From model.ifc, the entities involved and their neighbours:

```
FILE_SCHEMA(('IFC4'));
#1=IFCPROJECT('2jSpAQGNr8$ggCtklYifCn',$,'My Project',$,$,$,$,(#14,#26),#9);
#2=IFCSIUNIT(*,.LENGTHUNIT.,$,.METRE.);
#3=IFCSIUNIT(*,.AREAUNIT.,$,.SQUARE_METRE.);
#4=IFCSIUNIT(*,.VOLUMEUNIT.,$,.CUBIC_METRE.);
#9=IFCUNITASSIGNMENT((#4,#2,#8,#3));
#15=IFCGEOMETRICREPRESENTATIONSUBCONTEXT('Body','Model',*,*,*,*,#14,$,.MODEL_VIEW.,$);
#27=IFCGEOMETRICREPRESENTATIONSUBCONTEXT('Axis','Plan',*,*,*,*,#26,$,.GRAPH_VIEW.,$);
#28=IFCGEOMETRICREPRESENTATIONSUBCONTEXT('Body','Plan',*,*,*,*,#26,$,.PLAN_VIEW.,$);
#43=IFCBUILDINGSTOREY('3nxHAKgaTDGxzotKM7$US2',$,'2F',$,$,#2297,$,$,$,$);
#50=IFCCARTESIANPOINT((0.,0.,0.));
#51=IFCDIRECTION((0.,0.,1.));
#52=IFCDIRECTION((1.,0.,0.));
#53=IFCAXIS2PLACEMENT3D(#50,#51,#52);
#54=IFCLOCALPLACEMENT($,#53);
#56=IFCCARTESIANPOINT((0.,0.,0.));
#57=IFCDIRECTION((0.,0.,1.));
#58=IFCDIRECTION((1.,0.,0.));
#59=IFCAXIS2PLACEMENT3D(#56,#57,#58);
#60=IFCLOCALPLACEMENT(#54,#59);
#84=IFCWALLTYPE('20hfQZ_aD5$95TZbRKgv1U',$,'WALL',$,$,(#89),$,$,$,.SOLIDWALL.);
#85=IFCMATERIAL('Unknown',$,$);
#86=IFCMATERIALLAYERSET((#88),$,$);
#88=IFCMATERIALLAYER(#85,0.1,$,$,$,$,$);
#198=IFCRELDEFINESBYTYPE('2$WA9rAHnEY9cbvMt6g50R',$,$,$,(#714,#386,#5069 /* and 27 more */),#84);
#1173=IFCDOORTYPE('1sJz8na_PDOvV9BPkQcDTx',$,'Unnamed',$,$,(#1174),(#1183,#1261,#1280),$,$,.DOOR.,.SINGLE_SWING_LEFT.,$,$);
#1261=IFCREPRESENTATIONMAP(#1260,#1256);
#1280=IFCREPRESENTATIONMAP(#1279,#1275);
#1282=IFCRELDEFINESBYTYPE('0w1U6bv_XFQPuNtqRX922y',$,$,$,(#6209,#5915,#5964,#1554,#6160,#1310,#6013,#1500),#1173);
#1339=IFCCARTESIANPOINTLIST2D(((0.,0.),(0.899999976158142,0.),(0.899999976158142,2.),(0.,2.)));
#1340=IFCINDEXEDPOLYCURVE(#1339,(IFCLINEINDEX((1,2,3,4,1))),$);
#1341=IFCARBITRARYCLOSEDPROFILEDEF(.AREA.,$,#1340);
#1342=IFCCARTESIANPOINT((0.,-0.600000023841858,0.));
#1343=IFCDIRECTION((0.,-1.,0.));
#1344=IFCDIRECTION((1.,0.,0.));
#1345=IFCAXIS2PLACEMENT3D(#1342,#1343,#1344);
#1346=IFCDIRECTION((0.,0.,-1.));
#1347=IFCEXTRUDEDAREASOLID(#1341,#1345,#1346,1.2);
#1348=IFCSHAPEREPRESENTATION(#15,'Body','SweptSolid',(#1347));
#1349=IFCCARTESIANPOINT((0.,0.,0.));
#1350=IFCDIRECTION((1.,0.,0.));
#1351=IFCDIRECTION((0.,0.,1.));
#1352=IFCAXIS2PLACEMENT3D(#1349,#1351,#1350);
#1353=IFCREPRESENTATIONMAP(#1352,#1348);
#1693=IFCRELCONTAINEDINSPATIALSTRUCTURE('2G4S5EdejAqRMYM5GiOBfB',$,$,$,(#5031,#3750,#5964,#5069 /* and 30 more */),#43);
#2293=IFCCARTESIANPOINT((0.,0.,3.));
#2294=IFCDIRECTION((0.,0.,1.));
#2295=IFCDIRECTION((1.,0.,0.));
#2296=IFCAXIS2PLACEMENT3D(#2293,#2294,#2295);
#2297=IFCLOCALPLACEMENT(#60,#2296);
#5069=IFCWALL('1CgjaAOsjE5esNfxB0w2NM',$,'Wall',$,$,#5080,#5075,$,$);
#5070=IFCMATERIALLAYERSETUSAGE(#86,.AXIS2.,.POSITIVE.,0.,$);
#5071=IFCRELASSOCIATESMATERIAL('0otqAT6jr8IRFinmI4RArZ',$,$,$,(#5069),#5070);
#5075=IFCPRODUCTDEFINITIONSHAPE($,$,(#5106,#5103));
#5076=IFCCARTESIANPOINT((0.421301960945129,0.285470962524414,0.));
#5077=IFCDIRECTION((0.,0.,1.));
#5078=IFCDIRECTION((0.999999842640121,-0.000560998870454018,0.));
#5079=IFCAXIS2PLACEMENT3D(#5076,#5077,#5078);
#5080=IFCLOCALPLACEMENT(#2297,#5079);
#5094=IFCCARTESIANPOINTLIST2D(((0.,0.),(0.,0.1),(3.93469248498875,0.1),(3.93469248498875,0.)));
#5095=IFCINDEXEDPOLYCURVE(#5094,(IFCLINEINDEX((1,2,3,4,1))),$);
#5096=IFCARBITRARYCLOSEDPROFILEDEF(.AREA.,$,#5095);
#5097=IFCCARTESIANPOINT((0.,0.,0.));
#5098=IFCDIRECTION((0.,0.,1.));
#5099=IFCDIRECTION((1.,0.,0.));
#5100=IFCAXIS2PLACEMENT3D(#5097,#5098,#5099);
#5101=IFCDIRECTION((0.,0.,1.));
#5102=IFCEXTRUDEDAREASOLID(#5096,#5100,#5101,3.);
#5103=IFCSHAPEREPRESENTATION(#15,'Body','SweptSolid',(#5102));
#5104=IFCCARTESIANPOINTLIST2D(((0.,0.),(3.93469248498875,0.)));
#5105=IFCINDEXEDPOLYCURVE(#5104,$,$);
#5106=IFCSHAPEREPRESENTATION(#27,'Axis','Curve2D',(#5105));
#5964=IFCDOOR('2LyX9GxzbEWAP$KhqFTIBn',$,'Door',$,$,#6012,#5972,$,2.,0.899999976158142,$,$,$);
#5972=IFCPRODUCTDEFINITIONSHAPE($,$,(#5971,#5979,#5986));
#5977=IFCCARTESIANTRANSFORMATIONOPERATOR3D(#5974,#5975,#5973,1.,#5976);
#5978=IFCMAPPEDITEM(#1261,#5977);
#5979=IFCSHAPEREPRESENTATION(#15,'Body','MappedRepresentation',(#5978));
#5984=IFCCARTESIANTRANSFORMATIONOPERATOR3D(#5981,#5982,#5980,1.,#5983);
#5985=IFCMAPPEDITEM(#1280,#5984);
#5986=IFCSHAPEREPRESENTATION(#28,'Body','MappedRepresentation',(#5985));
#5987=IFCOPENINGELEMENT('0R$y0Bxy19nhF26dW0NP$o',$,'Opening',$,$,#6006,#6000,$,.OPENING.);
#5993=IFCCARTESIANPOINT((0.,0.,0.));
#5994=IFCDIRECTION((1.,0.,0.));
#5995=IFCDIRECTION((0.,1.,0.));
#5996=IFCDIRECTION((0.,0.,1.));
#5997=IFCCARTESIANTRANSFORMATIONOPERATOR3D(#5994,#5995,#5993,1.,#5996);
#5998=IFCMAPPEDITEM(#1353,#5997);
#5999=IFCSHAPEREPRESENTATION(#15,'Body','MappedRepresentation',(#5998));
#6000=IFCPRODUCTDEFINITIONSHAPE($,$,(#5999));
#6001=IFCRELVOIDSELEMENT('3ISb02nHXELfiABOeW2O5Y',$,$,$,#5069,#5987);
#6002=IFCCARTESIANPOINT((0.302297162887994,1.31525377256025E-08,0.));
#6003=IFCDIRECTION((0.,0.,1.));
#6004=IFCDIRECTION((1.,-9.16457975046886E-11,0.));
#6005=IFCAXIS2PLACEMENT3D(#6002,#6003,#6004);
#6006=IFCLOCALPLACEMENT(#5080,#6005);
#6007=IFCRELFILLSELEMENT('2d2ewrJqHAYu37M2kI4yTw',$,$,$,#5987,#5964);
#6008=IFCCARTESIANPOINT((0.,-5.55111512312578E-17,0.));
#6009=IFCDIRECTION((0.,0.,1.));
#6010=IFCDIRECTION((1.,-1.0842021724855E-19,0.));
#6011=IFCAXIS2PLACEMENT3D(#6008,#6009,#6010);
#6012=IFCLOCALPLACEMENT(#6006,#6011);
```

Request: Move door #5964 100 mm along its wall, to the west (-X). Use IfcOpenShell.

```python
import ifcopenshell
import ifcopenshell.api.geometry
import ifcopenshell.util.placement
import ifcopenshell.util.unit

model = ifcopenshell.open("model.ifc")
unit_scale = ifcopenshell.util.unit.calculate_unit_scale(model)

door = model.by_guid("2LyX9GxzbEWAP$KhqFTIBn")
opening = door.FillsVoids[0].RelatingOpeningElement
wall = opening.VoidsElements[0].RelatingBuildingElement

wall_matrix = ifcopenshell.util.placement.get_local_placement(wall.ObjectPlacement)
shift = wall_matrix[:3, 0] * -0.1 / unit_scale
before = ifcopenshell.util.placement.get_local_placement(door.ObjectPlacement)[:3, 3].copy()

# The door is placed relative to its opening, so it follows when the opening moves.
matrix = ifcopenshell.util.placement.get_local_placement(opening.ObjectPlacement)
matrix[:3, 3] += shift
ifcopenshell.api.geometry.edit_object_placement(
    model, product=opening, matrix=matrix, is_si=False, should_transform_children=True
)

after = ifcopenshell.util.placement.get_local_placement(door.ObjectPlacement)[:3, 3]
print("door moved by", (after - before).round(3) + 0.0)

model.write("model_updated.ifc")
```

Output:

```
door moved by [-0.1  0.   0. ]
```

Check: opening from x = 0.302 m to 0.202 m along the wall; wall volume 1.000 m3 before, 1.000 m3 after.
